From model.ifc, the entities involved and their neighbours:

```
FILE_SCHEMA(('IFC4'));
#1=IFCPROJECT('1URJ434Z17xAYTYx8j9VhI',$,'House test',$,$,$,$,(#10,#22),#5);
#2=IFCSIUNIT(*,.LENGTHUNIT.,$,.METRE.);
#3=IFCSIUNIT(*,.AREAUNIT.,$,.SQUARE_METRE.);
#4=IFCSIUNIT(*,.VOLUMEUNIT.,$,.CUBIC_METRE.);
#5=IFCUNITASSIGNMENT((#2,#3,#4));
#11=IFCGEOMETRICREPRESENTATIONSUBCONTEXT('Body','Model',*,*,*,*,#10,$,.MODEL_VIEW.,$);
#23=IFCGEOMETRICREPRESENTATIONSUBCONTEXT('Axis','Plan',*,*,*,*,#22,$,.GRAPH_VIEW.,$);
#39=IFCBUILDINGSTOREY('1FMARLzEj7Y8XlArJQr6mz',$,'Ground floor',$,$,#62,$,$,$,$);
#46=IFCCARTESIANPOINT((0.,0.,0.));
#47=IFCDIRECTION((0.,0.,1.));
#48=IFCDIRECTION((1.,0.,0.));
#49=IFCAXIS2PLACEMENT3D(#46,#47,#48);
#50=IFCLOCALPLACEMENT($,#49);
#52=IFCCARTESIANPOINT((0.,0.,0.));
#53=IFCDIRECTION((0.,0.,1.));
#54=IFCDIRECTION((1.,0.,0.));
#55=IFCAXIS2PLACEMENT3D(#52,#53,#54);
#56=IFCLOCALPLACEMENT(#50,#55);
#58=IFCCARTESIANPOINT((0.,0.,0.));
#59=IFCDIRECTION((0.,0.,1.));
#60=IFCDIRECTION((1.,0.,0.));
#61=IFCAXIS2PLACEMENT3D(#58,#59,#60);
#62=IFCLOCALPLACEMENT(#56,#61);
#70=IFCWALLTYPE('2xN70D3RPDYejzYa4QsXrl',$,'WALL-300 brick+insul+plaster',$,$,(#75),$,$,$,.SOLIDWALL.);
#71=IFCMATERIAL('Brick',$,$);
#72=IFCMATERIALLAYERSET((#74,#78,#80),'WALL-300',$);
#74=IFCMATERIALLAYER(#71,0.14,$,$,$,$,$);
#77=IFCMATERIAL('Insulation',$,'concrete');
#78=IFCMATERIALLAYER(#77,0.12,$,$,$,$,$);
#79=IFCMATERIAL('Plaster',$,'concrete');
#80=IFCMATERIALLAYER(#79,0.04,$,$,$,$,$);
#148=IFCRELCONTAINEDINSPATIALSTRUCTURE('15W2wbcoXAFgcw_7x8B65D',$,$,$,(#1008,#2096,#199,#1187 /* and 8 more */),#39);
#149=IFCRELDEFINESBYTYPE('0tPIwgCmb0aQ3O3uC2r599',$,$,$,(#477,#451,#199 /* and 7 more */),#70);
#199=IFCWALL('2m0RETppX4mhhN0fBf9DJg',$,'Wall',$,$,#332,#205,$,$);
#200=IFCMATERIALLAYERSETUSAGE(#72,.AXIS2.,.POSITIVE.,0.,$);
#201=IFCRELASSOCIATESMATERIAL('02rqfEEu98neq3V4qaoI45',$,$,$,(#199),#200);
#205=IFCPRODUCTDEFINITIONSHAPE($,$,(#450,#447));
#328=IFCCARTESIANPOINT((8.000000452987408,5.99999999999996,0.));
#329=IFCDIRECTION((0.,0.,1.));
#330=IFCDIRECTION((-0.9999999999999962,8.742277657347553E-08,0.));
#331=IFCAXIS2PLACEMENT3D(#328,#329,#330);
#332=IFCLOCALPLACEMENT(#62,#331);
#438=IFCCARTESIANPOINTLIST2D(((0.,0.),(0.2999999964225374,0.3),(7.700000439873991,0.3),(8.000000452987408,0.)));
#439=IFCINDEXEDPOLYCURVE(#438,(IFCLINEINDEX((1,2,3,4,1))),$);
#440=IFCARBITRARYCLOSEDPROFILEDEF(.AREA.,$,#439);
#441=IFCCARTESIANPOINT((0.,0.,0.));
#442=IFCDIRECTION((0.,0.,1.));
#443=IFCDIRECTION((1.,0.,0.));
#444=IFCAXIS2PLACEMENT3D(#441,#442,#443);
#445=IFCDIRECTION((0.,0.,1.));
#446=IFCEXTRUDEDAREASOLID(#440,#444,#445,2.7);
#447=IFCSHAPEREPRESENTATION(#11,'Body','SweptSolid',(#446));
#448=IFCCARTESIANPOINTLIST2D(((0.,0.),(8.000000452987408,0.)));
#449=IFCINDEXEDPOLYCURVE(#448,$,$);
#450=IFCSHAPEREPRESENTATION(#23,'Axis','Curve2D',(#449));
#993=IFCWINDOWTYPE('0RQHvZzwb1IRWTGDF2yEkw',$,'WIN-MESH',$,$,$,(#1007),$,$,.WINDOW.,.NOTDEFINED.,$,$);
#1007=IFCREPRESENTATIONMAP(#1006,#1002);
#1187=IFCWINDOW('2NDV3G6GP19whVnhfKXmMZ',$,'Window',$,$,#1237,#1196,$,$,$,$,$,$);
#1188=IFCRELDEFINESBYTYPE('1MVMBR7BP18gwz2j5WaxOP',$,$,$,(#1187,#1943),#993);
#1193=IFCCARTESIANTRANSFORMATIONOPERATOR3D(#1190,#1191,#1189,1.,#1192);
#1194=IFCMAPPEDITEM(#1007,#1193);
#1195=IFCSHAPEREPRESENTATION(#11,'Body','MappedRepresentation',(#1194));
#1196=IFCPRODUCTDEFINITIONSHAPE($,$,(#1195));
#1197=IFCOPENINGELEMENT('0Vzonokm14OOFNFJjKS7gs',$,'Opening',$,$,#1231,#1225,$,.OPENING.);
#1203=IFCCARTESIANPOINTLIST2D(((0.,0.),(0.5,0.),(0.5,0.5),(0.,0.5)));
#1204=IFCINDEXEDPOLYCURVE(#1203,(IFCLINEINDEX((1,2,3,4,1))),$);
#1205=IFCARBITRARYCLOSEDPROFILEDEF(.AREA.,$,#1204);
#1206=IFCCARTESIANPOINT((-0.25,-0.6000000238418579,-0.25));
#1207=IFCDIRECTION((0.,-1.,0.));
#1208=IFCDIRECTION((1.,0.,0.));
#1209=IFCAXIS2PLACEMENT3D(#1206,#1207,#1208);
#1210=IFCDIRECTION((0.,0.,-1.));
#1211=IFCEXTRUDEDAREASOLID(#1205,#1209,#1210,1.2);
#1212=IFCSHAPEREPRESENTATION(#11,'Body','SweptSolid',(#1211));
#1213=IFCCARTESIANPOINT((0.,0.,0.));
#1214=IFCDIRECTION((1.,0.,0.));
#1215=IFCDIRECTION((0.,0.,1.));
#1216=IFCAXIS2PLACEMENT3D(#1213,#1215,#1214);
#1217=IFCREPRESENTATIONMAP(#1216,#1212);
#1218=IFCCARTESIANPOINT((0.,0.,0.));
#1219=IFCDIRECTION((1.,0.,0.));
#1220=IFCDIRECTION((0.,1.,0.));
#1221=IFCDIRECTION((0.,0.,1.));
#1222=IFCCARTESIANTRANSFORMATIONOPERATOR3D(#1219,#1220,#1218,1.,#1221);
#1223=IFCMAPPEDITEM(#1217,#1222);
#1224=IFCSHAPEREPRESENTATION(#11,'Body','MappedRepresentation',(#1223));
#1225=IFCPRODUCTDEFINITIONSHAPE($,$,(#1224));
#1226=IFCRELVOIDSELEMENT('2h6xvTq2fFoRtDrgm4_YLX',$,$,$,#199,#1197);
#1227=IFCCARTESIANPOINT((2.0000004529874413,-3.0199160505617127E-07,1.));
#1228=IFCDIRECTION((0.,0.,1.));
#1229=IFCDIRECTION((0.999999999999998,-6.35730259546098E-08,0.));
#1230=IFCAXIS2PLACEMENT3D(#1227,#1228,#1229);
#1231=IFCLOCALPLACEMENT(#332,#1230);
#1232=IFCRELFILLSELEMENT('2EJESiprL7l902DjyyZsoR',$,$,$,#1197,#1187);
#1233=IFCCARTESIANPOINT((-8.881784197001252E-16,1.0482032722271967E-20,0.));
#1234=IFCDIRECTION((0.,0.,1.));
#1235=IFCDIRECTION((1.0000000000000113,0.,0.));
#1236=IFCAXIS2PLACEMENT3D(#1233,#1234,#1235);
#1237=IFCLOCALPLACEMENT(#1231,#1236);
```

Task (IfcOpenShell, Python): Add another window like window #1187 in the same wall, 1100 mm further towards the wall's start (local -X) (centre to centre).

```python
import ifcopenshell
import ifcopenshell.api.feature
import ifcopenshell.api.geometry
import ifcopenshell.api.root
import ifcopenshell.geom
import ifcopenshell.util.element
import ifcopenshell.util.placement
import ifcopenshell.util.shape
import ifcopenshell.util.unit

model = ifcopenshell.open("model.ifc")
unit_scale = ifcopenshell.util.unit.calculate_unit_scale(model)
settings = ifcopenshell.geom.settings()


def volume(element):
    """Net volume in cubic metres, openings subtracted."""
    shape = ifcopenshell.geom.create_shape(settings, element)
    return ifcopenshell.util.shape.get_volume(shape.geometry)


window = model.by_id(1187)
opening = window.FillsVoids[0].RelatingOpeningElement
wall = opening.VoidsElements[0].RelatingBuildingElement
before = volume(wall)
shift = ifcopenshell.util.placement.get_local_placement(wall.ObjectPlacement)[:3, 0] * -1.1 / unit_scale

# copy_class copies the void relationship, type, container and properties, but no geometry.
new_opening = ifcopenshell.api.root.copy_class(model, product=opening)
new_opening.Representation = ifcopenshell.util.element.copy_deep(
    model, opening.Representation, exclude=["IfcGeometricRepresentationContext", "IfcRepresentationMap"]
)
new_window = ifcopenshell.api.root.copy_class(model, product=window)
new_window.Representation = ifcopenshell.util.element.copy_deep(
    model, window.Representation, exclude=["IfcGeometricRepresentationContext", "IfcRepresentationMap"]
)
ifcopenshell.api.feature.add_filling(model, opening=new_opening, element=new_window)

for old, new in ((opening, new_opening), (window, new_window)):
    matrix = ifcopenshell.util.placement.get_local_placement(old.ObjectPlacement)
    matrix[:3, 3] += shift
    ifcopenshell.api.geometry.edit_object_placement(model, product=new, matrix=matrix, is_si=False)

after = volume(wall)

print(f"wall volume {before:.3f} -> {after:.3f} m3")

model.write("model_updated.ifc")
```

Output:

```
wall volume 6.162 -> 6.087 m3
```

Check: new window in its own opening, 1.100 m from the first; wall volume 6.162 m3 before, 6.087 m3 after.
